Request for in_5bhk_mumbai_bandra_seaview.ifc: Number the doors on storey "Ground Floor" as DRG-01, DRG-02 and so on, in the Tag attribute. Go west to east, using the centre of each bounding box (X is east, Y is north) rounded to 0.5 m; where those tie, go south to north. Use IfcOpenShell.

First a look at what the model holds.

```python
import ifcopenshell
import ifcopenshell.util.element
import ifcopenshell.util.placement

model = ifcopenshell.open("in_5bhk_mumbai_bandra_seaview.ifc")
print(model.schema)
storey = next(s for s in model.by_type("IfcBuildingStorey") if s.Name == "Ground Floor")
doors = [e for e in ifcopenshell.util.element.get_decomposition(storey) if e.is_a("IfcDoor")]
for e in sorted(doors, key=lambda e: e.id()):
    origin = ifcopenshell.util.placement.get_local_placement(e.ObjectPlacement)[:3, 3]
    print(e.id(), e.Tag, e.Name, origin.round(2) + 0.0, sep=" | ")
```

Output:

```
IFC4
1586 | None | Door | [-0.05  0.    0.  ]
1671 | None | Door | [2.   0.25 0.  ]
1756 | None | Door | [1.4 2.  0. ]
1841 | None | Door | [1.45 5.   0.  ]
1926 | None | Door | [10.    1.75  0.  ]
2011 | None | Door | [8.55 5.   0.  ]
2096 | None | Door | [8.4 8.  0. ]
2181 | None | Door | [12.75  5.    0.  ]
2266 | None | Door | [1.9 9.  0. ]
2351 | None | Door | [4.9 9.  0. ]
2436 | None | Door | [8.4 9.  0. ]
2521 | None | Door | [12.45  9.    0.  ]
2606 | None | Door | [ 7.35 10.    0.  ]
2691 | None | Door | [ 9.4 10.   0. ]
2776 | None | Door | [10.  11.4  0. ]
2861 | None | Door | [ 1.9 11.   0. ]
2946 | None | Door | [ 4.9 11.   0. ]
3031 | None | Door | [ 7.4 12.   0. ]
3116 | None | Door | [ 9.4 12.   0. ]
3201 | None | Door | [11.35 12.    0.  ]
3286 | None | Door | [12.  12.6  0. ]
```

```python
import ifcopenshell
import ifcopenshell.geom
import ifcopenshell.util.element
import ifcopenshell.util.shape

model = ifcopenshell.open("in_5bhk_mumbai_bandra_seaview.ifc")
settings = ifcopenshell.geom.settings()
settings.set("use-world-coords", True)


def centre(element):
    shape = ifcopenshell.geom.create_shape(settings, element)
    return ifcopenshell.util.shape.get_bbox_centroid(shape.geometry)


storey = next(s for s in model.by_type("IfcBuildingStorey") if s.Name == "Ground Floor")
doors = [e for e in ifcopenshell.util.element.get_decomposition(storey) if e.is_a("IfcDoor")]

# Insertion points can sit at a corner or the storey origin, so sort by the geometry (in metres).
centres = {e: centre(e) for e in doors}
doors.sort(key=lambda e: (round(centres[e][0] / 0.5), centres[e][1]))

for i, e in enumerate(doors, start=1):
    number = f"DRG-{i:02d}"
    e.Tag = number
    print(e.id(), number)

model.write("in_5bhk_mumbai_bandra_seaview_updated.ifc")
```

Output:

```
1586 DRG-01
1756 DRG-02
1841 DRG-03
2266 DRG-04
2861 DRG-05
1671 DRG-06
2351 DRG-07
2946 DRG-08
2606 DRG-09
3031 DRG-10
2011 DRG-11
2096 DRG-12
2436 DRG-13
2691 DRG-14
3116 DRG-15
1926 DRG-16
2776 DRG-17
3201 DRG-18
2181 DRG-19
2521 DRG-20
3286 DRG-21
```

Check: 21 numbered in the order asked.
